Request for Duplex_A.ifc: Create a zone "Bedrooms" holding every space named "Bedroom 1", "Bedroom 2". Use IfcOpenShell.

First a look at what the model holds.

```python
import ifcopenshell

model = ifcopenshell.open("Duplex_A.ifc")
print(model.schema)
seen = {}
for space in model.by_type("IfcSpace"):
    seen[space.LongName] = seen.get(space.LongName, 0) + 1
for name, count in sorted(seen.items(), key=str):
    print(count, "x", name)
print("zones:", [z.Name for z in model.by_type("IfcZone")][:20])
```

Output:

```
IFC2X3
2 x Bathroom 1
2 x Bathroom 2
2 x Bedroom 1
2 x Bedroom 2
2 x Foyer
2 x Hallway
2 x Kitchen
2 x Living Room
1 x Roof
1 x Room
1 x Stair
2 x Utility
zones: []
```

```python
import ifcopenshell
import ifcopenshell.api.group
import ifcopenshell.api.root

model = ifcopenshell.open("Duplex_A.ifc")

names = {"Bedroom 1", "Bedroom 2"}
spaces = [s for s in model.by_type("IfcSpace") if s.LongName in names]

zone = ifcopenshell.api.root.create_entity(model, ifc_class="IfcZone", name="Bedrooms")
ifcopenshell.api.group.assign_group(model, products=spaces, group=zone)
print(len(spaces), "spaces in", zone.Name)

model.write("Duplex_A_rev.ifc")
```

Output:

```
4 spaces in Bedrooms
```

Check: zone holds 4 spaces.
